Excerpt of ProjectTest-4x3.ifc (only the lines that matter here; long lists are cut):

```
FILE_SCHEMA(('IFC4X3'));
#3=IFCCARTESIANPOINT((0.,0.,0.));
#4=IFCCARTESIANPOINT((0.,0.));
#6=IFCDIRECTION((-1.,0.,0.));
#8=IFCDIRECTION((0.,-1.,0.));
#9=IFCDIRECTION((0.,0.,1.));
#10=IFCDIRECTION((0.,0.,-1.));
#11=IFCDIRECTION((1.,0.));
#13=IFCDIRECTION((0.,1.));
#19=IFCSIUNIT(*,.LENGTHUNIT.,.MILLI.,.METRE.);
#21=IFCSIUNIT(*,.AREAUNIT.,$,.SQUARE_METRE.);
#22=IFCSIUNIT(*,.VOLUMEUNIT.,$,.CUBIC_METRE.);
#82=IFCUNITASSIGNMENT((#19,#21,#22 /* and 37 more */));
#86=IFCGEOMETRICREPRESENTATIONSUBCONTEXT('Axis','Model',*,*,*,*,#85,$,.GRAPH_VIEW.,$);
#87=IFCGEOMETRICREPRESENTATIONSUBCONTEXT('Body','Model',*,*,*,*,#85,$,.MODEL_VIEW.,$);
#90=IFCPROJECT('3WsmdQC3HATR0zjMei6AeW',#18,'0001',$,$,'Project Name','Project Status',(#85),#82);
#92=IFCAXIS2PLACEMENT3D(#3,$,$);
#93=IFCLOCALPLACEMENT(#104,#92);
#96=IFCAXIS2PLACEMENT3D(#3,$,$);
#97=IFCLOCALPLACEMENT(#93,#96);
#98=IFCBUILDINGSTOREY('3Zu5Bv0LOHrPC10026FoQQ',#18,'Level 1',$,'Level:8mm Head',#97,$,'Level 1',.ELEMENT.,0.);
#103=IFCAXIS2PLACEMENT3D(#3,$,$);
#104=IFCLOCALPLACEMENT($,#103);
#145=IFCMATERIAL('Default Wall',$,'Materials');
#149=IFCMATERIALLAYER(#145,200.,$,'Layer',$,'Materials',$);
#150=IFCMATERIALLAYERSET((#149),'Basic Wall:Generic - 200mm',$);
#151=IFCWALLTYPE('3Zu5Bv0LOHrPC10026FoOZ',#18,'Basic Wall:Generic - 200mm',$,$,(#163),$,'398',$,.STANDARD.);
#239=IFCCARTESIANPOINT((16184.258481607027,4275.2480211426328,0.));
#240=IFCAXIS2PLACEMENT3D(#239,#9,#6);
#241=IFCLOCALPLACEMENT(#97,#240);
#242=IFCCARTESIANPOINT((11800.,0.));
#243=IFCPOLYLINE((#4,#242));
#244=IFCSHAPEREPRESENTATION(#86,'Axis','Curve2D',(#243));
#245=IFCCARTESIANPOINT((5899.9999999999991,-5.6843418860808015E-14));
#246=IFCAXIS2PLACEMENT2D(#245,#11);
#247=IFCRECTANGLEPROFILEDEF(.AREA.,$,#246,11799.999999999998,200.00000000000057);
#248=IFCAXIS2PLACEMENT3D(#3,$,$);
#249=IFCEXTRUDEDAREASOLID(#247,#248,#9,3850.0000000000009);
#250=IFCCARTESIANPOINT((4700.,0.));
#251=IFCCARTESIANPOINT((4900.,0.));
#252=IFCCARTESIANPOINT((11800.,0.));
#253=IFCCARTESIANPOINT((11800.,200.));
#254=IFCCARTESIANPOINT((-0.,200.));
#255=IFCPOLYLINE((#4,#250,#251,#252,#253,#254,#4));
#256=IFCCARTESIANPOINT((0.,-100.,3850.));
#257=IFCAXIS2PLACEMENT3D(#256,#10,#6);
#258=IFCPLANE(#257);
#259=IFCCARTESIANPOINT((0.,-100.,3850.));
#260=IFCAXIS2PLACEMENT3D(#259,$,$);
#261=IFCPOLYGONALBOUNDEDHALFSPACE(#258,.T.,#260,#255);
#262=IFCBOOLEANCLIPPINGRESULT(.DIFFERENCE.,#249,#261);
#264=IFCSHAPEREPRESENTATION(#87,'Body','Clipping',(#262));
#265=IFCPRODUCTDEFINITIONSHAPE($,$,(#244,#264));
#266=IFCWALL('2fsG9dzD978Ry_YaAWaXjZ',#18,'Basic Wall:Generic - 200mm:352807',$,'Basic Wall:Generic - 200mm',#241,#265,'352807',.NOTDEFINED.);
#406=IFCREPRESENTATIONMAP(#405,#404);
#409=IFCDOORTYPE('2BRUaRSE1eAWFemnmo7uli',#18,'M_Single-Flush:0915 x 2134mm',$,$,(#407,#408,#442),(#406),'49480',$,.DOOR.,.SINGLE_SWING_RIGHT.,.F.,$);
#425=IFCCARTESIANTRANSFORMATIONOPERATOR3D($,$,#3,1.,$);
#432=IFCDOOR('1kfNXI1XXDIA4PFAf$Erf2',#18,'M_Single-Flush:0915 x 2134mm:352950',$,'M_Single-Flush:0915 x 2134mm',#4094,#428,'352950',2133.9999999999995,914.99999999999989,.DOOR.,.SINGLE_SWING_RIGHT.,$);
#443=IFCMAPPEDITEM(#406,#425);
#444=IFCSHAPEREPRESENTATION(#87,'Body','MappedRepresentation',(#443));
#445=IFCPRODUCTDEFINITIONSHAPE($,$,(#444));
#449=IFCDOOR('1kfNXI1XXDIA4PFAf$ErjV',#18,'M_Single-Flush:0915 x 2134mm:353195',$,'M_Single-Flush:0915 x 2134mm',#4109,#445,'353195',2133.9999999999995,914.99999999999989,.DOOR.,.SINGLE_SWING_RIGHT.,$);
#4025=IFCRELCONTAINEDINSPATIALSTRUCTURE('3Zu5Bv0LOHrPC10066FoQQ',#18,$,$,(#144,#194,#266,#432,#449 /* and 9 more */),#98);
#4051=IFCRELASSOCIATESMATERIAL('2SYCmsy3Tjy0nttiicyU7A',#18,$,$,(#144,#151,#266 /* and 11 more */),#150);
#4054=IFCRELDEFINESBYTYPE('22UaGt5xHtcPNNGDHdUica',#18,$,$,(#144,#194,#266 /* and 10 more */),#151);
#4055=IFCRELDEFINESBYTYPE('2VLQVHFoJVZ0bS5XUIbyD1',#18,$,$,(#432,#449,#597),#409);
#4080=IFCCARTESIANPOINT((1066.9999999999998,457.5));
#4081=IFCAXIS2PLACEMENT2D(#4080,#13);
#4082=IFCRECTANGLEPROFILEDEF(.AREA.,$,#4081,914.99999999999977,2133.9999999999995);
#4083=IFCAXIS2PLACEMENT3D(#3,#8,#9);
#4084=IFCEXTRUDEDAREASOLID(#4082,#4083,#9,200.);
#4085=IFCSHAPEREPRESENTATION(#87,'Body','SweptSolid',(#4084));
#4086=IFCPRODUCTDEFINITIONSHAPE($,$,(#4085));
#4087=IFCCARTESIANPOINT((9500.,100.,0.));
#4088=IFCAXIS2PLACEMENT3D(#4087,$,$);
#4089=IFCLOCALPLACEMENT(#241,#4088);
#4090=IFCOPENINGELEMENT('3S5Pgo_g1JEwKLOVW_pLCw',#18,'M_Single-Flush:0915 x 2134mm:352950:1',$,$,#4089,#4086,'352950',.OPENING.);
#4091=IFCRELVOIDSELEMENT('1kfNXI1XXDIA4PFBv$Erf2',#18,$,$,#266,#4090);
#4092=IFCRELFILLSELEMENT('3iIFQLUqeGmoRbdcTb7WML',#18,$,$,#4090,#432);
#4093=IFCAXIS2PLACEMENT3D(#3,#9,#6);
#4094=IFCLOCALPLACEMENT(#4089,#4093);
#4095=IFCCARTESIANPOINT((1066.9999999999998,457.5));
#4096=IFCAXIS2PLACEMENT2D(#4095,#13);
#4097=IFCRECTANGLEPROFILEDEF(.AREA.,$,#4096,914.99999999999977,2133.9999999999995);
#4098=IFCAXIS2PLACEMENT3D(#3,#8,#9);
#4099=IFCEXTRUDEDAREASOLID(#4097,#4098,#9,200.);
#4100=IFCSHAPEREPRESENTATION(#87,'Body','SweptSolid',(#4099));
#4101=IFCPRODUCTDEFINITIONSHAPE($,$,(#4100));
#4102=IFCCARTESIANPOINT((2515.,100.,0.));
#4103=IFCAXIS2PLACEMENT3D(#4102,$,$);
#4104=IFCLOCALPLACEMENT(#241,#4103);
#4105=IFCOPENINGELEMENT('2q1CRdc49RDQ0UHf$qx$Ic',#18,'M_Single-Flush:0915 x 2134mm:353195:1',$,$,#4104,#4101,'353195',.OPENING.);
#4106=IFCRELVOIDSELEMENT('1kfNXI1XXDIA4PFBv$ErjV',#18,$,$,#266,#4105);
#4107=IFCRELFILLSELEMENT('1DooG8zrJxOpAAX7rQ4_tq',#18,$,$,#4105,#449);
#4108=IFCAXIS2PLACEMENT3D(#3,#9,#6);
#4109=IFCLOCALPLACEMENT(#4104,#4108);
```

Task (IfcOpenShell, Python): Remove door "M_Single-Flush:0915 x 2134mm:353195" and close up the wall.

```python
import ifcopenshell
import ifcopenshell.api.feature
import ifcopenshell.api.root
import ifcopenshell.geom
import ifcopenshell.util.shape

model = ifcopenshell.open("ProjectTest-4x3.ifc")
settings = ifcopenshell.geom.settings()


def volume(element):
    """Net volume in cubic metres, openings subtracted."""
    shape = ifcopenshell.geom.create_shape(settings, element)
    return ifcopenshell.util.shape.get_volume(shape.geometry)


door = model.by_guid("1kfNXI1XXDIA4PFAf$ErjV")
opening = door.FillsVoids[0].RelatingOpeningElement
wall = opening.VoidsElements[0].RelatingBuildingElement
before = volume(wall)

ifcopenshell.api.root.remove_product(model, product=door)
ifcopenshell.api.feature.remove_feature(model, feature=opening)

after = volume(wall)

print(f"wall volume {before:.3f} -> {after:.3f} m3")

model.write("ProjectTest-4x3_rev.ifc")
```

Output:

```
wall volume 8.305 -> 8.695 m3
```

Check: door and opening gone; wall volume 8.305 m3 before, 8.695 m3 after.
